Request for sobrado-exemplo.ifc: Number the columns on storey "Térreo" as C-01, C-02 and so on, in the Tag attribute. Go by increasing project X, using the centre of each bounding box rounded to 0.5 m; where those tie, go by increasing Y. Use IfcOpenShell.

First a look at what the model holds.

```python
import ifcopenshell
import ifcopenshell.util.element
import ifcopenshell.util.placement

model = ifcopenshell.open("sobrado-exemplo.ifc")
print(model.schema)
storey = next(s for s in model.by_type("IfcBuildingStorey") if s.Name == "Térreo")
columns = [e for e in ifcopenshell.util.element.get_decomposition(storey) if e.is_a("IfcColumn")]
for e in sorted(columns, key=lambda e: e.id()):
    origin = ifcopenshell.util.placement.get_local_placement(e.ObjectPlacement)[:3, 3]
    print(e.id(), e.Tag, e.Name, origin.round(2) + 0.0, sep=" | ")
```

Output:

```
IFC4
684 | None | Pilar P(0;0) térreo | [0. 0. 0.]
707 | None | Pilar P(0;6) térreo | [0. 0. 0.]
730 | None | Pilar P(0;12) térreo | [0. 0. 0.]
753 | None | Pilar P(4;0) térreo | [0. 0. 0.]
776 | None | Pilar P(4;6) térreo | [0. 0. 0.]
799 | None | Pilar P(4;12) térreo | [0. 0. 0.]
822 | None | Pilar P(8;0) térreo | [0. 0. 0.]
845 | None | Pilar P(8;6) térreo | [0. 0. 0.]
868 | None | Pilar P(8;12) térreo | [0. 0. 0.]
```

```python
import ifcopenshell
import ifcopenshell.geom
import ifcopenshell.util.element
import ifcopenshell.util.shape

model = ifcopenshell.open("sobrado-exemplo.ifc")
settings = ifcopenshell.geom.settings()
settings.set("use-world-coords", True)


def centre(element):
    shape = ifcopenshell.geom.create_shape(settings, element)
    return ifcopenshell.util.shape.get_bbox_centroid(shape.geometry)


storey = next(s for s in model.by_type("IfcBuildingStorey") if s.Name == "Térreo")
columns = [e for e in ifcopenshell.util.element.get_decomposition(storey) if e.is_a("IfcColumn")]

# Insertion points can sit at a corner or the storey origin, so sort by the geometry (in metres).
centres = {e: centre(e) for e in columns}
columns.sort(key=lambda e: (round(centres[e][0] / 0.5), centres[e][1]))

for i, e in enumerate(columns, start=1):
    number = f"C-{i:02d}"
    e.Tag = number
    print(e.id(), number)

model.write("sobrado-exemplo-out.ifc")
```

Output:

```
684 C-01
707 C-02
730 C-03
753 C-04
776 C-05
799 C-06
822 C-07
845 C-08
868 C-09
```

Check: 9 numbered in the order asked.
